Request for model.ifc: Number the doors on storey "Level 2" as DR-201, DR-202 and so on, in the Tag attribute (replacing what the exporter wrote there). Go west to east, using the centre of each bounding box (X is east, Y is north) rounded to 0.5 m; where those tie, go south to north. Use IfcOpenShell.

First a look at what the model holds.

```python
import ifcopenshell
import ifcopenshell.util.element
import ifcopenshell.util.placement

model = ifcopenshell.open("model.ifc")
print(model.schema)
storey = next(s for s in model.by_type("IfcBuildingStorey") if s.Name == "Level 2")
doors = [e for e in ifcopenshell.util.element.get_decomposition(storey) if e.is_a("IfcDoor")]
for e in sorted(doors, key=lambda e: e.id()):
    origin = ifcopenshell.util.placement.get_local_placement(e.ObjectPlacement)[:3, 3]
    print(e.id(), e.Tag, e.Name, origin.round(2) + 0.0, sep=" | ")
```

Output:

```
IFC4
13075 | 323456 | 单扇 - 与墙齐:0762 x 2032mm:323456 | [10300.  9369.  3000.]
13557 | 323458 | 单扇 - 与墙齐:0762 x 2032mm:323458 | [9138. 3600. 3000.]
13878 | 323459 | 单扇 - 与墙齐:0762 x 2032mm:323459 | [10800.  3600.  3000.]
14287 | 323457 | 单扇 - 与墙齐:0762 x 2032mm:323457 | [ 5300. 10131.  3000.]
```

```python
import ifcopenshell
import ifcopenshell.geom
import ifcopenshell.util.element
import ifcopenshell.util.shape

model = ifcopenshell.open("model.ifc")
settings = ifcopenshell.geom.settings()
settings.set("use-world-coords", True)


def centre(element):
    shape = ifcopenshell.geom.create_shape(settings, element)
    return ifcopenshell.util.shape.get_bbox_centroid(shape.geometry)


storey = next(s for s in model.by_type("IfcBuildingStorey") if s.Name == "Level 2")
doors = [e for e in ifcopenshell.util.element.get_decomposition(storey) if e.is_a("IfcDoor")]

# Insertion points can sit at a corner or the storey origin, so sort by the geometry (in metres).
centres = {e: centre(e) for e in doors}
doors.sort(key=lambda e: (round(centres[e][0] / 0.5), centres[e][1]))

for i, e in enumerate(doors, start=1):
    number = f"DR-2{i:02d}"
    e.Tag = number
    print(e.id(), number)

model.write("model_v2.ifc")
```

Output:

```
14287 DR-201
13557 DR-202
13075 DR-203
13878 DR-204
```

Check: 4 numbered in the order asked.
